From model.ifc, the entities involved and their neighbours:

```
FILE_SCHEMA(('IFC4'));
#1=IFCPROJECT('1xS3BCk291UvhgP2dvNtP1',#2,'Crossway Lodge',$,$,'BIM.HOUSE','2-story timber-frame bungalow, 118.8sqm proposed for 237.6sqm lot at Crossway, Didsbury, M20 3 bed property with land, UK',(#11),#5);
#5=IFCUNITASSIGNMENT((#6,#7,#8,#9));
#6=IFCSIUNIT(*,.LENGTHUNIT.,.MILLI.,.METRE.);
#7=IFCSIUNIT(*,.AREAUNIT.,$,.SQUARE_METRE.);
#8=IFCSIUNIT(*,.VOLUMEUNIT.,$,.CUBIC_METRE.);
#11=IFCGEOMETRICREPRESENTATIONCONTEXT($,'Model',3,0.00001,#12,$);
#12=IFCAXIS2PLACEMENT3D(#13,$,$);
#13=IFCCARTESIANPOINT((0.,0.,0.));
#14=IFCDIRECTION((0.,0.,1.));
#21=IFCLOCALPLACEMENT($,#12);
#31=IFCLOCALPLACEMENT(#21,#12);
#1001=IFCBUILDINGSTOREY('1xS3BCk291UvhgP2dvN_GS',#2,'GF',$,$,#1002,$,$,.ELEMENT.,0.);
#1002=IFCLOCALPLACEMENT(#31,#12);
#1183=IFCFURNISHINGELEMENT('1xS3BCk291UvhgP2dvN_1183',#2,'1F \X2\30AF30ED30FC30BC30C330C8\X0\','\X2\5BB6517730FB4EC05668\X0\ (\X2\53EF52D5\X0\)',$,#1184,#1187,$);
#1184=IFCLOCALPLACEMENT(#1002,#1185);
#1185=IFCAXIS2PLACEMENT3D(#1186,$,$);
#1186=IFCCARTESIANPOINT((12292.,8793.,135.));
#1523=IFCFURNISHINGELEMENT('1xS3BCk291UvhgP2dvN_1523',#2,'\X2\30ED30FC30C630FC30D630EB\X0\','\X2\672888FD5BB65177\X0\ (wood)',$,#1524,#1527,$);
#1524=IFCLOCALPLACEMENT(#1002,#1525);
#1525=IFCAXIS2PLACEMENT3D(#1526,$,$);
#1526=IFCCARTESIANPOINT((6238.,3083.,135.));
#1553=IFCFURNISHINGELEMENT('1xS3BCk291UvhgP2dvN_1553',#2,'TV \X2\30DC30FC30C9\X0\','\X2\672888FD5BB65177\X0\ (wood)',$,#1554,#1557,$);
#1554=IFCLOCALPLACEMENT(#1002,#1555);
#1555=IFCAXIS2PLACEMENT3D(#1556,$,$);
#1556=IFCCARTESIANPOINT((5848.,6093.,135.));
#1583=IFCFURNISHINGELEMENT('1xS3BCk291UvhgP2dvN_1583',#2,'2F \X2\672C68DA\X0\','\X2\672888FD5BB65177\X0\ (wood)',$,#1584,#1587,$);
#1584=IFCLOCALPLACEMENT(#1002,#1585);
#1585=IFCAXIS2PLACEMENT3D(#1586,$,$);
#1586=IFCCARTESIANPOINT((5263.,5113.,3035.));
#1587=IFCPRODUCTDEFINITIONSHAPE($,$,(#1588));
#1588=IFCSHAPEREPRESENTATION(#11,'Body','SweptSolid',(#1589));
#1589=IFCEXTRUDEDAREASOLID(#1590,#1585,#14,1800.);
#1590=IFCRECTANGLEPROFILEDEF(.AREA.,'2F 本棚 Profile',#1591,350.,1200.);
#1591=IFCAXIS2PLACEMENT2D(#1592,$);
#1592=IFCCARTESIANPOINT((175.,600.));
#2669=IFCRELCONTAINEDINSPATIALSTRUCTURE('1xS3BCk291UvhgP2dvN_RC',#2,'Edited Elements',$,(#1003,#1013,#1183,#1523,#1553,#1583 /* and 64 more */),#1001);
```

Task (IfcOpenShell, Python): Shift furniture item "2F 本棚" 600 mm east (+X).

```python
import ifcopenshell
import ifcopenshell.api.geometry
import ifcopenshell.util.placement
import ifcopenshell.util.unit

model = ifcopenshell.open("model.ifc")
unit_scale = ifcopenshell.util.unit.calculate_unit_scale(model)

item = model.by_id(1583)
matrix = ifcopenshell.util.placement.get_local_placement(item.ObjectPlacement)
matrix[0, 3] += 0.6 / unit_scale
ifcopenshell.api.geometry.edit_object_placement(model, product=item, matrix=matrix, is_si=False)

print(ifcopenshell.util.placement.get_local_placement(item.ObjectPlacement).round(3) + 0.0)

model.write("model-out.ifc")
```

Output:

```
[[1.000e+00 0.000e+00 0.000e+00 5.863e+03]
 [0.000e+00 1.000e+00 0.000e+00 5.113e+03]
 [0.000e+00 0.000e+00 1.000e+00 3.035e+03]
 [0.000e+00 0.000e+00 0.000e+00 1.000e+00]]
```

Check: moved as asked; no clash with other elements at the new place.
